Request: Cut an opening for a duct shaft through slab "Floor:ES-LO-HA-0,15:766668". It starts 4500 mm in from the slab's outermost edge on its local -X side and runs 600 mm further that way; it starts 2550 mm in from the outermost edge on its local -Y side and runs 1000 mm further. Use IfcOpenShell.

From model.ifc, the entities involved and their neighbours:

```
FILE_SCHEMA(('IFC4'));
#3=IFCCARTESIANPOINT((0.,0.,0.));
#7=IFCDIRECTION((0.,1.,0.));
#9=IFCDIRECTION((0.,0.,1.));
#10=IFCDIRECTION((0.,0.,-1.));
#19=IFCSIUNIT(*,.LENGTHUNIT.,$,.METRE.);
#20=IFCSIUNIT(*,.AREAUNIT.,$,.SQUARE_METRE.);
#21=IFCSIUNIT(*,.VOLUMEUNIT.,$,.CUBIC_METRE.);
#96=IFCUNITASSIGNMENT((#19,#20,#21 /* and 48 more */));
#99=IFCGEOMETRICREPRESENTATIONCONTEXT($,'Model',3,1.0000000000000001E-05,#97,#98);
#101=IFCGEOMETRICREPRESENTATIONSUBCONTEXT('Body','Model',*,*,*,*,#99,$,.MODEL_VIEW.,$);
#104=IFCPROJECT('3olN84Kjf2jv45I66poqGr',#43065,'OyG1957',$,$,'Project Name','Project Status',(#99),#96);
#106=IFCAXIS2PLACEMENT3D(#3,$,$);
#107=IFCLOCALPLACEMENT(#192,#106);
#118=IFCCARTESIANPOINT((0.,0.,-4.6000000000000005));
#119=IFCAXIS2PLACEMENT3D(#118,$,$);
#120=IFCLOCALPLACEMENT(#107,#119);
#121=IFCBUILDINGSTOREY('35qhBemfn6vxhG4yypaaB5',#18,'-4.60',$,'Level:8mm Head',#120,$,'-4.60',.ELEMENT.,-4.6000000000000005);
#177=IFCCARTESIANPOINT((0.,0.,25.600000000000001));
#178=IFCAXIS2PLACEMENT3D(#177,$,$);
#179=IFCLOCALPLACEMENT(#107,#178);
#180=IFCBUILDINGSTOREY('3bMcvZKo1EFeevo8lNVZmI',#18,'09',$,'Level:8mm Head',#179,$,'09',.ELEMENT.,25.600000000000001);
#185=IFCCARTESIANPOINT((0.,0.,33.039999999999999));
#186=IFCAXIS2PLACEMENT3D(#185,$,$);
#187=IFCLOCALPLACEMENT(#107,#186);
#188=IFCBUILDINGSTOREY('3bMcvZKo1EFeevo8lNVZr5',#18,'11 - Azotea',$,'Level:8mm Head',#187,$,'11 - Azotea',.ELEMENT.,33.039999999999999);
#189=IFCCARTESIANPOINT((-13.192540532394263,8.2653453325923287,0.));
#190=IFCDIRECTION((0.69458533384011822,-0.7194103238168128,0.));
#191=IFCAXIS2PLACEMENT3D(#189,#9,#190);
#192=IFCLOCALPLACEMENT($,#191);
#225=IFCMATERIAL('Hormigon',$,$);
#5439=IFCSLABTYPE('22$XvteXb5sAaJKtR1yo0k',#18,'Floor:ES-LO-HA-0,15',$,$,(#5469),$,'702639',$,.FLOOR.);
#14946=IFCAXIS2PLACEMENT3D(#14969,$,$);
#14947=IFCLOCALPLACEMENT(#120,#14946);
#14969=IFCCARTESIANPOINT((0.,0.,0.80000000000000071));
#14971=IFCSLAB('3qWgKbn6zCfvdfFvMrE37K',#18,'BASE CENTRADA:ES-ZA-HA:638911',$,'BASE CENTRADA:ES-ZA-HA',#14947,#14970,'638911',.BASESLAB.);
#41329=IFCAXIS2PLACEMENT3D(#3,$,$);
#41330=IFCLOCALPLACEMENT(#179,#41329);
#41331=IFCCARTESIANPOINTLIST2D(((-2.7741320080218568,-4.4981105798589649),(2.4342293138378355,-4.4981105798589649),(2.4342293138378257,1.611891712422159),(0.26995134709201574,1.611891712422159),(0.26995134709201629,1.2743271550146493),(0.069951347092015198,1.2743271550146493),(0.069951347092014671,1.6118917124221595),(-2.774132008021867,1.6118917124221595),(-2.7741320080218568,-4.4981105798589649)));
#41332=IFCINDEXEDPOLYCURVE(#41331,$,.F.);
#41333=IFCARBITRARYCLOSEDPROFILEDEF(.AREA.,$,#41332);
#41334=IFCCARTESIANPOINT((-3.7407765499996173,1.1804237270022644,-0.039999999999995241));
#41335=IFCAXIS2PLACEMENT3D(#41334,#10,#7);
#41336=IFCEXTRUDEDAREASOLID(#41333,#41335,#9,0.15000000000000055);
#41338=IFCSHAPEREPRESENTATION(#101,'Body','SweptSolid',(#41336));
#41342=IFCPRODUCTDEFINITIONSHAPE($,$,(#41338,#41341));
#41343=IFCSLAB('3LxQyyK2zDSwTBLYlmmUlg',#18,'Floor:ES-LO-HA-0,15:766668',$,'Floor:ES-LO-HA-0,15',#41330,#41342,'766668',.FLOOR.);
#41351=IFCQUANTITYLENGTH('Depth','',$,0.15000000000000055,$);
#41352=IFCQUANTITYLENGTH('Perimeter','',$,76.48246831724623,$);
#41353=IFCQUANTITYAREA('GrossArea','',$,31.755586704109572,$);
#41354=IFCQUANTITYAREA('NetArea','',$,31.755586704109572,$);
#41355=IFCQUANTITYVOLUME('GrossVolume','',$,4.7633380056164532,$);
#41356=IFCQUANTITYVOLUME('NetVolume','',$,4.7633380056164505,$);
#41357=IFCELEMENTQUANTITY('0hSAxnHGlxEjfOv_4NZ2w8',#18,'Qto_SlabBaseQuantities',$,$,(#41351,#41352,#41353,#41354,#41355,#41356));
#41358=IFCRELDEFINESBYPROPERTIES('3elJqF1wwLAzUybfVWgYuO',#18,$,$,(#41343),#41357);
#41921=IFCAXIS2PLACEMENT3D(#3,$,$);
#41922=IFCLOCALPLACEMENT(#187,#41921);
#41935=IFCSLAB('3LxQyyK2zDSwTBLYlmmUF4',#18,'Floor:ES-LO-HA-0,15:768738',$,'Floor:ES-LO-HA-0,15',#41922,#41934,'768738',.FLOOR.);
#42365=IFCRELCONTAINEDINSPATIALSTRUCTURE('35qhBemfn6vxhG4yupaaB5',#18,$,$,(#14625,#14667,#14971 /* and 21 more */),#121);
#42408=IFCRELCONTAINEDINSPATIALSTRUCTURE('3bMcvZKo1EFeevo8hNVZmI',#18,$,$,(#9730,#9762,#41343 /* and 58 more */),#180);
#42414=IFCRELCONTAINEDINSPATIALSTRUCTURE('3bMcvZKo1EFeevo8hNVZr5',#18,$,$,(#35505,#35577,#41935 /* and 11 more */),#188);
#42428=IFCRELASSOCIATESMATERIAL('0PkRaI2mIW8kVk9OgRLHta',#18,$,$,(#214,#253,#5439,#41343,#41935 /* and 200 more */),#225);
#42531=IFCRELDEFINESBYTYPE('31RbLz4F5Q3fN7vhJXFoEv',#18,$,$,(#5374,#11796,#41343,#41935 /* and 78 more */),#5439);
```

```python
import numpy as np
import ifcopenshell
import ifcopenshell.api.feature
import ifcopenshell.api.geometry
import ifcopenshell.api.pset
import ifcopenshell.api.root
import ifcopenshell.geom
import ifcopenshell.util.element
import ifcopenshell.util.placement
import ifcopenshell.util.representation
import ifcopenshell.util.shape
import ifcopenshell.util.unit

model = ifcopenshell.open("model.ifc")
unit_scale = ifcopenshell.util.unit.calculate_unit_scale(model)
area_scale = ifcopenshell.util.unit.calculate_unit_scale(model, "AREAUNIT")
volume_scale = ifcopenshell.util.unit.calculate_unit_scale(model, "VOLUMEUNIT")
settings = ifcopenshell.geom.settings()


def volume(element):
    """Net volume in cubic metres, openings subtracted."""
    shape = ifcopenshell.geom.create_shape(settings, element)
    return ifcopenshell.util.shape.get_volume(shape.geometry)


slab = model.by_id(41343)
before = volume(slab)

# Extent in the slab's own axes, in metres. The edges named are its -X and -Y sides.
slab_shape = ifcopenshell.geom.create_shape(settings, slab)
vertices = ifcopenshell.util.shape.get_vertices(slab_shape.geometry)
x_min, y_min, bottom = vertices.min(axis=0)
top = vertices[:, 2].max()

opening = ifcopenshell.api.root.create_entity(model, ifc_class="IfcOpeningElement", name="Duct shaft opening", predefined_type="OPENING")
context = ifcopenshell.util.representation.get_context(model, "Model", "Body", "MODEL_VIEW")
width, depth = 0.6, 1
outline = [(0.0, 0.0), (width, 0.0), (width, depth), (0.0, depth), (0.0, 0.0)]
# Overshoot both faces by 50 mm so the cut is clean.
shape = ifcopenshell.api.geometry.add_slab_representation(
    model, context=context, depth=top - bottom + 0.1, polyline=outline
)
ifcopenshell.api.geometry.assign_representation(model, product=opening, representation=shape)

matrix = ifcopenshell.util.placement.get_local_placement(slab.ObjectPlacement)
matrix[:, 3] = matrix @ np.append(np.array([x_min + 4.5, y_min + 2.55, bottom - 0.05]) / unit_scale, 1.0)
ifcopenshell.api.geometry.edit_object_placement(model, product=opening, matrix=matrix, is_si=False)
ifcopenshell.api.feature.add_feature(model, feature=opening, element=slab)

after = volume(slab)

# Update the slab's stored quantities.
qto = model.by_id(ifcopenshell.util.element.get_pset(slab, "Qto_SlabBaseQuantities", should_inherit=False)["id"])
ifcopenshell.api.pset.edit_qto(model, qto=qto, properties={
    "NetArea": after / (top - bottom) / area_scale,
    "NetVolume": after / volume_scale,
})

print(f"slab volume {before:.3f} -> {after:.3f} m3")

model.write("model-out.ifc")
```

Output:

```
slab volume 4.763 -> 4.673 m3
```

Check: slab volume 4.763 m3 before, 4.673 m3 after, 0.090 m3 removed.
